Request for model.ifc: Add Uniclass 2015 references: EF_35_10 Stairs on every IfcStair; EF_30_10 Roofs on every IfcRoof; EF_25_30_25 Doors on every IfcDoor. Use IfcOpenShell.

First a look at what the model holds.

```python
import ifcopenshell

model = ifcopenshell.open("model.ifc")
print(model.schema)
print("classifications:", [c.Name for c in model.by_type("IfcClassification")])
for ifc_class in ("IfcDoor", "IfcRoof", "IfcStair", "IfcWall", "IfcWindow"):
    print(ifc_class, len(model.by_type(ifc_class)))
```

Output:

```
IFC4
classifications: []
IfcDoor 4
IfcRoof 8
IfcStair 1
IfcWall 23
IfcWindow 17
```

```python
import ifcopenshell
import ifcopenshell.api.classification

model = ifcopenshell.open("model.ifc")

system = ifcopenshell.api.classification.add_classification(model, classification="Uniclass 2015")

codes = {
    "IfcStair": ("EF_35_10", "Stairs"),
    "IfcRoof": ("EF_30_10", "Roofs"),
    "IfcDoor": ("EF_25_30_25", "Doors"),
}
for ifc_class, (code, name) in codes.items():
    products = model.by_type(ifc_class)
    ifcopenshell.api.classification.add_reference(
        model, products=products, classification=system, identification=code, name=name
    )
    print(code, len(products))

model.write("model_rev.ifc")
```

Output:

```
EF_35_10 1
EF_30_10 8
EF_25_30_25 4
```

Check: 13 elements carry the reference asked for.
